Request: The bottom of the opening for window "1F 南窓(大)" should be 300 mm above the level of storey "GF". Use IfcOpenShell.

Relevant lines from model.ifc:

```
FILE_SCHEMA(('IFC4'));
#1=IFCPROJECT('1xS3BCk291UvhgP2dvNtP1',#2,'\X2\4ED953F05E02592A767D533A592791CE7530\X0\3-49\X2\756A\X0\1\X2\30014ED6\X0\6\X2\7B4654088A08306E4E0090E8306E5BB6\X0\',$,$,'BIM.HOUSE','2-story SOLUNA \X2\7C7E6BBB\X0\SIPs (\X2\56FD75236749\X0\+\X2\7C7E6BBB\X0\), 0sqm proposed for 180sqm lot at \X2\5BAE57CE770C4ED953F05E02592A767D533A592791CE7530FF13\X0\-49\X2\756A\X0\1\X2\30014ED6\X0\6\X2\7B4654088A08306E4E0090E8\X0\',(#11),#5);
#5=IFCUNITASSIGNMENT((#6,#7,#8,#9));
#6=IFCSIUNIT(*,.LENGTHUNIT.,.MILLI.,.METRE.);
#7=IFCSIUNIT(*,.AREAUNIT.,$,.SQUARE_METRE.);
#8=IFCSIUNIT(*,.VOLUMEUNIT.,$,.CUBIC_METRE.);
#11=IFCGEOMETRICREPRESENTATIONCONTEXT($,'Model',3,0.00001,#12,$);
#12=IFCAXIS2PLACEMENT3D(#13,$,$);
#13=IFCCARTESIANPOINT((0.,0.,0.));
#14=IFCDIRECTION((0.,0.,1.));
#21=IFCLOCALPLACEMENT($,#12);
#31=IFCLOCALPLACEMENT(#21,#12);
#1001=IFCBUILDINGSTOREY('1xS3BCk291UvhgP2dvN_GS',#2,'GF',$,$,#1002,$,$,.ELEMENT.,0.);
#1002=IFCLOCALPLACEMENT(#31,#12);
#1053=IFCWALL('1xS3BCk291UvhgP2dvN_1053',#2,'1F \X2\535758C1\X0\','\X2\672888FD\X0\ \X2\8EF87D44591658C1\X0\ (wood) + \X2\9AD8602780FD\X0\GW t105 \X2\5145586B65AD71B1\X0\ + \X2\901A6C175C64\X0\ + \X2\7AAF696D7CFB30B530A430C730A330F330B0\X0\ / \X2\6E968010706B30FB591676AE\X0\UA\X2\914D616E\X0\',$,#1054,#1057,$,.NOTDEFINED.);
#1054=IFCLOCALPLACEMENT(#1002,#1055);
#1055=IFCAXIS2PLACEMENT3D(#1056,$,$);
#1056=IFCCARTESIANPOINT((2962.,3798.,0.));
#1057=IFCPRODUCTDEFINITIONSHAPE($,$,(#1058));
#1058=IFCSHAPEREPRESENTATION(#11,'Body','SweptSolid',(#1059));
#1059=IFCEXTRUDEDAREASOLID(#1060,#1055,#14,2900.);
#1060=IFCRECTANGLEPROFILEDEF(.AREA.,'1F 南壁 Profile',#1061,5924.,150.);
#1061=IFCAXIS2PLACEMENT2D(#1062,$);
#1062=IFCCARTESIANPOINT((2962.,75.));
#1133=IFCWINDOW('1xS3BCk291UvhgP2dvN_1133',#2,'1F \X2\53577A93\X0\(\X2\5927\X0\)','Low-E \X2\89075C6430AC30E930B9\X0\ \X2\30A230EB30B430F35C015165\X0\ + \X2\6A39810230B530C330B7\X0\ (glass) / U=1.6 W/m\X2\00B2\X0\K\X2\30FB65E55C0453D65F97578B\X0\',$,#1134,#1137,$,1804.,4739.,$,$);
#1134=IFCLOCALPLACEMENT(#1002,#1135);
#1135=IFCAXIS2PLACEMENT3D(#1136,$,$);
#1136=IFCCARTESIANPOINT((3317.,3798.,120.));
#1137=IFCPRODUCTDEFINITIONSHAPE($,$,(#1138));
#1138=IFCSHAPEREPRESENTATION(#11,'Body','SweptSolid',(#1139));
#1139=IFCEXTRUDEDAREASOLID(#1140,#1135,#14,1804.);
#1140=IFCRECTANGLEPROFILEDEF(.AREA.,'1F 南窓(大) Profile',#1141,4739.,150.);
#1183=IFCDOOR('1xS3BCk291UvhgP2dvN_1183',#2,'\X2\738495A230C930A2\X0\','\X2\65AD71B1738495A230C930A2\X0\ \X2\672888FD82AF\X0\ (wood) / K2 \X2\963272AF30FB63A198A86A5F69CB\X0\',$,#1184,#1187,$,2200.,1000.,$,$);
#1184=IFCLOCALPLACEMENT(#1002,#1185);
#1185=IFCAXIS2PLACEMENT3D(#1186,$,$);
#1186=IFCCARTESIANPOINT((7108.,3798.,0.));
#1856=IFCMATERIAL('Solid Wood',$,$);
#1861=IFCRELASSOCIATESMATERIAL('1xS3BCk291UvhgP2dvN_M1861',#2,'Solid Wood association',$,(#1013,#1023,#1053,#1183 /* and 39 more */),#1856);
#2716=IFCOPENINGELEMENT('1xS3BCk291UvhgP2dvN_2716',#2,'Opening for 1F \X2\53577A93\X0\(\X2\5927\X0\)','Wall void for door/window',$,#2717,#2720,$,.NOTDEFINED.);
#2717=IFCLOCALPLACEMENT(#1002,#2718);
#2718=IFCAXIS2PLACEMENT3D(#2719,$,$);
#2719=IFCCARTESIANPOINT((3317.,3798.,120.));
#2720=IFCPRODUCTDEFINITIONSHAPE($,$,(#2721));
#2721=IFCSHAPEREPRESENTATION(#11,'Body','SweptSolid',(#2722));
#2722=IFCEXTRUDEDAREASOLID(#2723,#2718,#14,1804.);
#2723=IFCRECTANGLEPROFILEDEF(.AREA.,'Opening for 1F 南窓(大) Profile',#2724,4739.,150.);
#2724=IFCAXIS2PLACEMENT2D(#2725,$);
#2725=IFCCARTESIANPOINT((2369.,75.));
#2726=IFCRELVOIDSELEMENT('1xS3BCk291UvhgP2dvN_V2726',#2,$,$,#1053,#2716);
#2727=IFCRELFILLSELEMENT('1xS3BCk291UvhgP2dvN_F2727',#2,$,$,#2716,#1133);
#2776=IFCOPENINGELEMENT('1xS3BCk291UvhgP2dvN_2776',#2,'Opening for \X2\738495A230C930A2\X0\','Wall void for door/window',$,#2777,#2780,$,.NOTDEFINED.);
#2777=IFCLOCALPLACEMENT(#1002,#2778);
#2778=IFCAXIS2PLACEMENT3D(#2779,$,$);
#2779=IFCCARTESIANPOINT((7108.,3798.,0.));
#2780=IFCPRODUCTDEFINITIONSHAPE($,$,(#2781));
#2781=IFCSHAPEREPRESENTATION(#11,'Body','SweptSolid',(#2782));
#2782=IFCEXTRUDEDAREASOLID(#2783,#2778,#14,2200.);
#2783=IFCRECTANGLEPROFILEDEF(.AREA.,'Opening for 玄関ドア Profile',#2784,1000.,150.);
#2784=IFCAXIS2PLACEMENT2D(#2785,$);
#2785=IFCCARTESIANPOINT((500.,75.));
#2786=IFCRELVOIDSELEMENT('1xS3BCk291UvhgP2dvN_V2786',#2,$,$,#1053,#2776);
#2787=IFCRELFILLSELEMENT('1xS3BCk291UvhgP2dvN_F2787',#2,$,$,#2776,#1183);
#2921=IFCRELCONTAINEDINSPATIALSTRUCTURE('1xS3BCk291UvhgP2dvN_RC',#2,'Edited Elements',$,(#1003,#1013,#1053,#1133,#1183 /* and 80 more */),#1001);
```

```python
import numpy as np
import ifcopenshell
import ifcopenshell.api.geometry
import ifcopenshell.geom
import ifcopenshell.util.element
import ifcopenshell.util.placement
import ifcopenshell.util.shape
import ifcopenshell.util.unit

model = ifcopenshell.open("model.ifc")
unit_scale = ifcopenshell.util.unit.calculate_unit_scale(model)

window = model.by_id(1133)
opening = window.FillsVoids[0].RelatingOpeningElement
storey = ifcopenshell.util.element.get_container(window, ifc_class="IfcBuildingStorey")
level = ifcopenshell.util.placement.get_local_placement(storey.ObjectPlacement)[2, 3]

# The opening's origin need not be at the sill, so measure its lowest point.
shape = ifcopenshell.geom.create_shape(ifcopenshell.geom.settings(), opening)
bottom = ifcopenshell.util.shape.get_shape_bottom_elevation(shape, shape.geometry) / unit_scale
dz = level + 300.0 - bottom

shift = np.array([0.0, 0.0, dz])
# The window is not placed relative to its opening, so move both.
for product in (opening, window):
    matrix = ifcopenshell.util.placement.get_local_placement(product.ObjectPlacement)
    matrix[:3, 3] += shift
    ifcopenshell.api.geometry.edit_object_placement(model, product=product, matrix=matrix, is_si=False)

print(f"moved by {dz * unit_scale:+.3f} m")

model.write("model-out.ifc")
```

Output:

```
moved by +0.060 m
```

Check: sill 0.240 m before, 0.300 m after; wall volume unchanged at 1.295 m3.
